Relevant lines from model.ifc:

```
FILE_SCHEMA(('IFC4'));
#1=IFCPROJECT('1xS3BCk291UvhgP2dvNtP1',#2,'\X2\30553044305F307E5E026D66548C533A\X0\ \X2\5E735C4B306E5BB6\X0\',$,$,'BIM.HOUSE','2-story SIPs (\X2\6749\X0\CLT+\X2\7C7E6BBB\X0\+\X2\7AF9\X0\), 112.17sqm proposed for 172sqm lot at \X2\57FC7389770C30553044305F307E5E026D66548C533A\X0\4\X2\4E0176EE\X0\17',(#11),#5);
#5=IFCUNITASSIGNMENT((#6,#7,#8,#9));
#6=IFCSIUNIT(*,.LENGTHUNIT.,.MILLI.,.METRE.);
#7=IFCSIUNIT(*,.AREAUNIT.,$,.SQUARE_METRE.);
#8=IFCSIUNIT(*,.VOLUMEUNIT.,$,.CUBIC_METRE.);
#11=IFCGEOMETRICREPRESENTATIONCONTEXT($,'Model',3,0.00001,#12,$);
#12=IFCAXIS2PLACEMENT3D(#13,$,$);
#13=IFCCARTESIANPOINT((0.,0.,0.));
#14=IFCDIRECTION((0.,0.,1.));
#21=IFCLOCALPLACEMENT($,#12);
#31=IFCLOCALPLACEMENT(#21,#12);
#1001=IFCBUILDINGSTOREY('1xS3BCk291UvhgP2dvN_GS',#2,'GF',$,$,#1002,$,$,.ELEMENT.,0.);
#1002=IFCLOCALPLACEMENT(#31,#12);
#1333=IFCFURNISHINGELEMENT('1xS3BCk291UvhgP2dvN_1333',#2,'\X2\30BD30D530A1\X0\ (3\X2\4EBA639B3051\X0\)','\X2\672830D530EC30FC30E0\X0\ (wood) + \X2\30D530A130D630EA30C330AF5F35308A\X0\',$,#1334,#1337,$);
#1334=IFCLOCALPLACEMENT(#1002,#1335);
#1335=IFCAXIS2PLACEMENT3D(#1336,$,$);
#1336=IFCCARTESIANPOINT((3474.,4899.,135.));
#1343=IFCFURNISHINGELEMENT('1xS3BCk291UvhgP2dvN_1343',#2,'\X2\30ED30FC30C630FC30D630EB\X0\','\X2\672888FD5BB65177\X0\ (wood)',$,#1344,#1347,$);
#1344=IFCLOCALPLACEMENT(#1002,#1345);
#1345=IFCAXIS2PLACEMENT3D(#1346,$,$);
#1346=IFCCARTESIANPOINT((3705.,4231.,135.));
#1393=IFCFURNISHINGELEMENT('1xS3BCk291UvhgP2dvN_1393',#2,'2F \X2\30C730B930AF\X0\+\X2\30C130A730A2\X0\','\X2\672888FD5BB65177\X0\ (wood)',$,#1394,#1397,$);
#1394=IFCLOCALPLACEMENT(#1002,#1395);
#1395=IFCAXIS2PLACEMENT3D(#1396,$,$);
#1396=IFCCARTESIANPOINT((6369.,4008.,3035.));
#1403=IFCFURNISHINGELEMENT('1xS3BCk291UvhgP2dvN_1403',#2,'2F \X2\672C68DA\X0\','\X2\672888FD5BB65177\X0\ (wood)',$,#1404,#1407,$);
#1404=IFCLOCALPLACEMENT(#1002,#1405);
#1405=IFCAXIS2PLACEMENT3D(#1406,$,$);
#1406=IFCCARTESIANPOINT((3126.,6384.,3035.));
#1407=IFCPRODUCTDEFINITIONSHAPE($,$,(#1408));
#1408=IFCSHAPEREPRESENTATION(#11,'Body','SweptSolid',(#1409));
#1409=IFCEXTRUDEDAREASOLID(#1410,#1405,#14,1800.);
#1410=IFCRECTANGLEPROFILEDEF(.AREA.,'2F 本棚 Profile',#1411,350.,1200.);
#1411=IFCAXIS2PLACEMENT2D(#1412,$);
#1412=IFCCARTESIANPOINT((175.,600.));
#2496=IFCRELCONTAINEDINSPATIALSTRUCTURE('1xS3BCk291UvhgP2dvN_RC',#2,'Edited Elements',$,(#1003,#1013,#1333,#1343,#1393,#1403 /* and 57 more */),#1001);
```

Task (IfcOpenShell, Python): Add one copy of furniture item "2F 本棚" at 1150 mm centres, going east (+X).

```python
import numpy as np
import ifcopenshell
import ifcopenshell.api.geometry
import ifcopenshell.api.root
import ifcopenshell.util.element
import ifcopenshell.util.placement
import ifcopenshell.util.unit

model = ifcopenshell.open("model.ifc")
unit_scale = ifcopenshell.util.unit.calculate_unit_scale(model)


def reuse_history(source, copy):
    """copy_class also copies each property set's owner history, people and application; keep the originals."""
    for rel in copy.IsDefinedBy:
        if rel.is_a("IfcRelDefinesByProperties") and (history := rel.RelatingPropertyDefinition.OwnerHistory):
            rel.RelatingPropertyDefinition.OwnerHistory = source.OwnerHistory
            ifcopenshell.util.element.remove_deep2(model, history)


source = model.by_guid("1xS3BCk291UvhgP2dvN_1403")
base = ifcopenshell.util.placement.get_local_placement(source.ObjectPlacement)
step = np.array([1.0, 0.0, 0.0]) * 1.15 / unit_scale

for i in range(1, 2):
    copy = ifcopenshell.api.root.copy_class(model, product=source)
    copy.Representation = ifcopenshell.util.element.copy_deep(
        model, source.Representation, exclude=["IfcGeometricRepresentationContext", "IfcRepresentationMap"]
    )
    reuse_history(source, copy)
    matrix = base.copy()
    matrix[:3, 3] += i * step
    print("added at", matrix[:3, 3].round(3) + 0.0)
    ifcopenshell.api.geometry.edit_object_placement(model, product=copy, matrix=matrix, is_si=False)

model.write("model_updated.ifc")
```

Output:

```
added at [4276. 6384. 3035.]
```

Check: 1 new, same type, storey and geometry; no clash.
